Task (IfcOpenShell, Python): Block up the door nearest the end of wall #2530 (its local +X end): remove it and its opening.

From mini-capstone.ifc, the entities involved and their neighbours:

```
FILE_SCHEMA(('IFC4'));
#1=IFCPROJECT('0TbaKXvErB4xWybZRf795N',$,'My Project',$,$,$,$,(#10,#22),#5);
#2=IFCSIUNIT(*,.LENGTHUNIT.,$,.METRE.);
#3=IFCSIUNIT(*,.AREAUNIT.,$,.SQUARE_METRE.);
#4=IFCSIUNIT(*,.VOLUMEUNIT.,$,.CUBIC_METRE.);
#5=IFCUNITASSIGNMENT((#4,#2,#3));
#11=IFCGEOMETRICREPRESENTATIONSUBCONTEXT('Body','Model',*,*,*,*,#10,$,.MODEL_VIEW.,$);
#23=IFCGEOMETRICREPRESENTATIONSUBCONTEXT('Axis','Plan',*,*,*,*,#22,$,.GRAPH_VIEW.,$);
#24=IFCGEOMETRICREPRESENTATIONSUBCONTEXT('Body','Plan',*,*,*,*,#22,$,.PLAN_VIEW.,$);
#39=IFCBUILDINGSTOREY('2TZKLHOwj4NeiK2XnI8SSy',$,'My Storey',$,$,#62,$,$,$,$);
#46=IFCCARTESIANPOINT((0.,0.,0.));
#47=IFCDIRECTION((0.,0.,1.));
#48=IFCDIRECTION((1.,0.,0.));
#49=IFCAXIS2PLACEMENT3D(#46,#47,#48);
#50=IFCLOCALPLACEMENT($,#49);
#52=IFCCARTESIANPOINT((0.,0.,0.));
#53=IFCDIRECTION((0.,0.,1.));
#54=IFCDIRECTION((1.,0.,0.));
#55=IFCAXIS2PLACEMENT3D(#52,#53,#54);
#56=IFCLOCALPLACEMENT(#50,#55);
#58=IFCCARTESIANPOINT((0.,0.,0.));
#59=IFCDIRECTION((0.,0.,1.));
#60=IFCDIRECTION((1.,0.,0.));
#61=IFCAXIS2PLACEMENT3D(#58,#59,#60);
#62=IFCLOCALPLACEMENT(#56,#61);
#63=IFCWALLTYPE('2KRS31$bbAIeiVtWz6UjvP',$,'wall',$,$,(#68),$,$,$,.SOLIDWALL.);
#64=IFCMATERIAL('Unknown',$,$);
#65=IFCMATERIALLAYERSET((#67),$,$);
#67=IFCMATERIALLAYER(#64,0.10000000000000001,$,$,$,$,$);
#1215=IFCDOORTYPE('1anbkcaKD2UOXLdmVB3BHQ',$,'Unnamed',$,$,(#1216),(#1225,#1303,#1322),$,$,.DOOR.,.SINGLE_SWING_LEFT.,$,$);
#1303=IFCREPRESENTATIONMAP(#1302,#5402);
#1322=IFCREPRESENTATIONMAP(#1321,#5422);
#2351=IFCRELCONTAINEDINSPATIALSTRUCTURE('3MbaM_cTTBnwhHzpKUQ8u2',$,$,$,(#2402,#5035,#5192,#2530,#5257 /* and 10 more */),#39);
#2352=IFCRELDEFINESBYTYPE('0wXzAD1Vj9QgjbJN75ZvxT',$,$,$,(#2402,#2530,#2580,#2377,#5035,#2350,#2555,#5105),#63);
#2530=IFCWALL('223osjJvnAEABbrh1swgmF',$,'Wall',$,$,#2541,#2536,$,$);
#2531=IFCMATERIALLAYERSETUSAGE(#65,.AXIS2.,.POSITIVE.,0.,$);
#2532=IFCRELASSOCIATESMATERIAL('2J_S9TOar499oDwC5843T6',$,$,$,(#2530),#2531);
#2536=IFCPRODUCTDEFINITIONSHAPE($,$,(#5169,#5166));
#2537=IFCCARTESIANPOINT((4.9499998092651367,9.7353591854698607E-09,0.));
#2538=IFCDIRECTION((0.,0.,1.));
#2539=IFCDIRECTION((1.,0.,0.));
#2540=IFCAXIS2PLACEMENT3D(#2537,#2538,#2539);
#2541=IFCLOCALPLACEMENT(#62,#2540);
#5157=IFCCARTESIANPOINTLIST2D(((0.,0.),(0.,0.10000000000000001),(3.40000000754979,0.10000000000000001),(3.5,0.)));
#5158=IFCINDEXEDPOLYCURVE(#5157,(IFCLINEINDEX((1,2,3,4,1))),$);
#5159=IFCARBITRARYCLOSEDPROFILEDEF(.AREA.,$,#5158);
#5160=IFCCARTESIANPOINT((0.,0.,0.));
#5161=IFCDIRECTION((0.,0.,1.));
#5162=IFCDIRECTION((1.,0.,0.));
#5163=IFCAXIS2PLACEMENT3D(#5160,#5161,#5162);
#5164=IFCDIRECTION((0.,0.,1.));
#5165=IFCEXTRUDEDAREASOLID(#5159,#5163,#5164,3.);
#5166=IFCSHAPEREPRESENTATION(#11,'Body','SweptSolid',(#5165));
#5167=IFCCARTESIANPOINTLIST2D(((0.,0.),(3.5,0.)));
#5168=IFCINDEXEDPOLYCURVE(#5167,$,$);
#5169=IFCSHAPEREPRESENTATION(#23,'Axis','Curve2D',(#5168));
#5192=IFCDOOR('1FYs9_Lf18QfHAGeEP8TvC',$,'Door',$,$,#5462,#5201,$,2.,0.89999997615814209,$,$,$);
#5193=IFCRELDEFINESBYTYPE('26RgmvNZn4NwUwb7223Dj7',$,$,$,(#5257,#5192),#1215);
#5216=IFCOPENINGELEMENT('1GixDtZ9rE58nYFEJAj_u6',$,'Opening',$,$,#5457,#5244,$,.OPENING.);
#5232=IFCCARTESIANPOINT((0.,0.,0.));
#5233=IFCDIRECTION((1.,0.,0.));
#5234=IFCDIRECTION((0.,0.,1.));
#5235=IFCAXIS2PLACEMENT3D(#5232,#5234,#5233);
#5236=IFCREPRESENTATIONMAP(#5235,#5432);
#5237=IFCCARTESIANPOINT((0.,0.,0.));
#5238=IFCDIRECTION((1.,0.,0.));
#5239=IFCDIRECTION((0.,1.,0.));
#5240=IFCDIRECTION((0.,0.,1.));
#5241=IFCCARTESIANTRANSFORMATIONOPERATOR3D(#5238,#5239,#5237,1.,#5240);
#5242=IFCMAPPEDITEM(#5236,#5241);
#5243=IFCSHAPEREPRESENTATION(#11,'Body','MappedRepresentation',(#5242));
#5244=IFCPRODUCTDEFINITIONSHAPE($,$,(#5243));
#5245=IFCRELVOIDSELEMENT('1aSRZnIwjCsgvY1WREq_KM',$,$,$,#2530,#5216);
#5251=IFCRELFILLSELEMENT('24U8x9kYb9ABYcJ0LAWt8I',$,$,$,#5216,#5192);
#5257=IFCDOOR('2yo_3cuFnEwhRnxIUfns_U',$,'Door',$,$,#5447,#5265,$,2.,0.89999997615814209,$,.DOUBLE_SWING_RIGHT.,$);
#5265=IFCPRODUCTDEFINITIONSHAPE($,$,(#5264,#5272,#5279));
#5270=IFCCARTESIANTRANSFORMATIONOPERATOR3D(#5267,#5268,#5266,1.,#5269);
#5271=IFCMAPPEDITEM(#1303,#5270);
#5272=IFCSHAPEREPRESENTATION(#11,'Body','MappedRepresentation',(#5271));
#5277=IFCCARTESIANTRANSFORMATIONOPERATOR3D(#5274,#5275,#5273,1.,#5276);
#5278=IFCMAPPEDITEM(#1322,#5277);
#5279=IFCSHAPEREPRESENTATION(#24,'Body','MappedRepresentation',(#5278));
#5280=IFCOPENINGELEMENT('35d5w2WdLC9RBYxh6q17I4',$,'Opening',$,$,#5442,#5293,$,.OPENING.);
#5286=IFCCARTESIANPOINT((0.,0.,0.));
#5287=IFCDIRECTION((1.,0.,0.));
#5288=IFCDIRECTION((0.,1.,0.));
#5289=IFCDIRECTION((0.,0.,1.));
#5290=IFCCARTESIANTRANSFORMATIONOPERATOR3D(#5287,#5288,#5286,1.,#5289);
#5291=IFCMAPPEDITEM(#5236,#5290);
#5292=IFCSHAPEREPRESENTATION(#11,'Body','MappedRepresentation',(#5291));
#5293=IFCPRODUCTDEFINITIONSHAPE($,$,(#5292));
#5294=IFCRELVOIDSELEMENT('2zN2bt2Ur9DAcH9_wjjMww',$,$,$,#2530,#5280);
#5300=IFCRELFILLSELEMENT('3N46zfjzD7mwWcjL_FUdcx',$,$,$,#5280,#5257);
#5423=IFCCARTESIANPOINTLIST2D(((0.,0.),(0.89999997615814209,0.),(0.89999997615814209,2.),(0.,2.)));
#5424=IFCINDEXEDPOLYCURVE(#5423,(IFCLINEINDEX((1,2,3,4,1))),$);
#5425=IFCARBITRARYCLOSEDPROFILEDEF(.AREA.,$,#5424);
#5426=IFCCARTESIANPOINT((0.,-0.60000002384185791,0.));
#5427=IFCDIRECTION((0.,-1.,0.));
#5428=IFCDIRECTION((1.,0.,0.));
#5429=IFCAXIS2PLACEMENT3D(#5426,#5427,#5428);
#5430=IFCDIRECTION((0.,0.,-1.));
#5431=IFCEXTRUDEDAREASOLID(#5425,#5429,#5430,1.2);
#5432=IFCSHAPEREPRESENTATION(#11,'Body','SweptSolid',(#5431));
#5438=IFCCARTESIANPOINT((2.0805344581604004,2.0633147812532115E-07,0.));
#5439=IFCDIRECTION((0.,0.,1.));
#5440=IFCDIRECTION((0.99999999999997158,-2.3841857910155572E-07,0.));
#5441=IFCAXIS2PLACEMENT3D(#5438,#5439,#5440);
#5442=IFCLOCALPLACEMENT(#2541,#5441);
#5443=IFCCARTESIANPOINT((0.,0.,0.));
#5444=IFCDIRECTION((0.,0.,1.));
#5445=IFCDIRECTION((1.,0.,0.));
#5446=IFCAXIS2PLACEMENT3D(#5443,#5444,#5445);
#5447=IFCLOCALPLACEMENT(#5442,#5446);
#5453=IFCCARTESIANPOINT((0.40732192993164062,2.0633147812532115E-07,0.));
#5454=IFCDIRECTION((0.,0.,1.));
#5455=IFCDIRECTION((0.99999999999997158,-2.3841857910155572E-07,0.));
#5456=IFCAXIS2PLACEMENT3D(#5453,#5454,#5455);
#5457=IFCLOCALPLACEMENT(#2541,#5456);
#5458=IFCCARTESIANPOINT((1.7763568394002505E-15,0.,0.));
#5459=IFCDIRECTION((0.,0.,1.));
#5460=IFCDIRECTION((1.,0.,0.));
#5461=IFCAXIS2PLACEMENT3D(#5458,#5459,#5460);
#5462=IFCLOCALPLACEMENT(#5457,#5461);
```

```python
import ifcopenshell
import ifcopenshell.api.feature
import ifcopenshell.api.root
import ifcopenshell.geom
import ifcopenshell.util.shape

model = ifcopenshell.open("mini-capstone.ifc")
settings = ifcopenshell.geom.settings()


def volume(element):
    """Net volume in cubic metres, openings subtracted."""
    shape = ifcopenshell.geom.create_shape(settings, element)
    return ifcopenshell.util.shape.get_volume(shape.geometry)


door = model.by_guid("2yo_3cuFnEwhRnxIUfns_U")
opening = door.FillsVoids[0].RelatingOpeningElement
wall = opening.VoidsElements[0].RelatingBuildingElement
before = volume(wall)

ifcopenshell.api.root.remove_product(model, product=door)
ifcopenshell.api.feature.remove_feature(model, feature=opening)

after = volume(wall)

print(f"wall volume {before:.3f} -> {after:.3f} m3")

model.write("mini-capstone_v2.ifc")
```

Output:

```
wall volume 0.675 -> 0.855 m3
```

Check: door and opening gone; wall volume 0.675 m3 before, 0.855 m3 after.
